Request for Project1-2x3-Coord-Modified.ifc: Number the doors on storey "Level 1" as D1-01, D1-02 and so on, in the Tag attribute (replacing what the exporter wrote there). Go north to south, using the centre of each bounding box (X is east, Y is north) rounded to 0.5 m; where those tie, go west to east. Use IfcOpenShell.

First a look at what the model holds.

```python
import ifcopenshell
import ifcopenshell.util.element
import ifcopenshell.util.placement

model = ifcopenshell.open("Project1-2x3-Coord-Modified.ifc")
print(model.schema)
storey = next(s for s in model.by_type("IfcBuildingStorey") if s.Name == "Level 1")
doors = [e for e in ifcopenshell.util.element.get_decomposition(storey) if e.is_a("IfcDoor")]
for e in sorted(doors, key=lambda e: e.id()):
    origin = ifcopenshell.util.placement.get_local_placement(e.ObjectPlacement)[:3, 3]
    print(e.id(), e.Tag, e.Name, origin.round(2) + 0.0, sep=" | ")
```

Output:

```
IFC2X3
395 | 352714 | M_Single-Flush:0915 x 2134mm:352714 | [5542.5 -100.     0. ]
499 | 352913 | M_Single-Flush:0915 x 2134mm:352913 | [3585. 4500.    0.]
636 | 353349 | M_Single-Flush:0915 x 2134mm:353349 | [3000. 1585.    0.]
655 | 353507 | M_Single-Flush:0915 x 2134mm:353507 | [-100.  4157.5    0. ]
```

```python
import ifcopenshell
import ifcopenshell.geom
import ifcopenshell.util.element
import ifcopenshell.util.shape

model = ifcopenshell.open("Project1-2x3-Coord-Modified.ifc")
settings = ifcopenshell.geom.settings()
settings.set("use-world-coords", True)


def centre(element):
    shape = ifcopenshell.geom.create_shape(settings, element)
    return ifcopenshell.util.shape.get_bbox_centroid(shape.geometry)


storey = next(s for s in model.by_type("IfcBuildingStorey") if s.Name == "Level 1")
doors = [e for e in ifcopenshell.util.element.get_decomposition(storey) if e.is_a("IfcDoor")]

# Insertion points can sit at a corner or the storey origin, so sort by the geometry (in metres).
centres = {e: centre(e) for e in doors}
doors.sort(key=lambda e: (-round(centres[e][1] / 0.5), centres[e][0]))

for i, e in enumerate(doors, start=1):
    number = f"D1-{i:02d}"
    e.Tag = number
    print(e.id(), number)

model.write("Project1-2x3-Coord-Modified_v2.ifc")
```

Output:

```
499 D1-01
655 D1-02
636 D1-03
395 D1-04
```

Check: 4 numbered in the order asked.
